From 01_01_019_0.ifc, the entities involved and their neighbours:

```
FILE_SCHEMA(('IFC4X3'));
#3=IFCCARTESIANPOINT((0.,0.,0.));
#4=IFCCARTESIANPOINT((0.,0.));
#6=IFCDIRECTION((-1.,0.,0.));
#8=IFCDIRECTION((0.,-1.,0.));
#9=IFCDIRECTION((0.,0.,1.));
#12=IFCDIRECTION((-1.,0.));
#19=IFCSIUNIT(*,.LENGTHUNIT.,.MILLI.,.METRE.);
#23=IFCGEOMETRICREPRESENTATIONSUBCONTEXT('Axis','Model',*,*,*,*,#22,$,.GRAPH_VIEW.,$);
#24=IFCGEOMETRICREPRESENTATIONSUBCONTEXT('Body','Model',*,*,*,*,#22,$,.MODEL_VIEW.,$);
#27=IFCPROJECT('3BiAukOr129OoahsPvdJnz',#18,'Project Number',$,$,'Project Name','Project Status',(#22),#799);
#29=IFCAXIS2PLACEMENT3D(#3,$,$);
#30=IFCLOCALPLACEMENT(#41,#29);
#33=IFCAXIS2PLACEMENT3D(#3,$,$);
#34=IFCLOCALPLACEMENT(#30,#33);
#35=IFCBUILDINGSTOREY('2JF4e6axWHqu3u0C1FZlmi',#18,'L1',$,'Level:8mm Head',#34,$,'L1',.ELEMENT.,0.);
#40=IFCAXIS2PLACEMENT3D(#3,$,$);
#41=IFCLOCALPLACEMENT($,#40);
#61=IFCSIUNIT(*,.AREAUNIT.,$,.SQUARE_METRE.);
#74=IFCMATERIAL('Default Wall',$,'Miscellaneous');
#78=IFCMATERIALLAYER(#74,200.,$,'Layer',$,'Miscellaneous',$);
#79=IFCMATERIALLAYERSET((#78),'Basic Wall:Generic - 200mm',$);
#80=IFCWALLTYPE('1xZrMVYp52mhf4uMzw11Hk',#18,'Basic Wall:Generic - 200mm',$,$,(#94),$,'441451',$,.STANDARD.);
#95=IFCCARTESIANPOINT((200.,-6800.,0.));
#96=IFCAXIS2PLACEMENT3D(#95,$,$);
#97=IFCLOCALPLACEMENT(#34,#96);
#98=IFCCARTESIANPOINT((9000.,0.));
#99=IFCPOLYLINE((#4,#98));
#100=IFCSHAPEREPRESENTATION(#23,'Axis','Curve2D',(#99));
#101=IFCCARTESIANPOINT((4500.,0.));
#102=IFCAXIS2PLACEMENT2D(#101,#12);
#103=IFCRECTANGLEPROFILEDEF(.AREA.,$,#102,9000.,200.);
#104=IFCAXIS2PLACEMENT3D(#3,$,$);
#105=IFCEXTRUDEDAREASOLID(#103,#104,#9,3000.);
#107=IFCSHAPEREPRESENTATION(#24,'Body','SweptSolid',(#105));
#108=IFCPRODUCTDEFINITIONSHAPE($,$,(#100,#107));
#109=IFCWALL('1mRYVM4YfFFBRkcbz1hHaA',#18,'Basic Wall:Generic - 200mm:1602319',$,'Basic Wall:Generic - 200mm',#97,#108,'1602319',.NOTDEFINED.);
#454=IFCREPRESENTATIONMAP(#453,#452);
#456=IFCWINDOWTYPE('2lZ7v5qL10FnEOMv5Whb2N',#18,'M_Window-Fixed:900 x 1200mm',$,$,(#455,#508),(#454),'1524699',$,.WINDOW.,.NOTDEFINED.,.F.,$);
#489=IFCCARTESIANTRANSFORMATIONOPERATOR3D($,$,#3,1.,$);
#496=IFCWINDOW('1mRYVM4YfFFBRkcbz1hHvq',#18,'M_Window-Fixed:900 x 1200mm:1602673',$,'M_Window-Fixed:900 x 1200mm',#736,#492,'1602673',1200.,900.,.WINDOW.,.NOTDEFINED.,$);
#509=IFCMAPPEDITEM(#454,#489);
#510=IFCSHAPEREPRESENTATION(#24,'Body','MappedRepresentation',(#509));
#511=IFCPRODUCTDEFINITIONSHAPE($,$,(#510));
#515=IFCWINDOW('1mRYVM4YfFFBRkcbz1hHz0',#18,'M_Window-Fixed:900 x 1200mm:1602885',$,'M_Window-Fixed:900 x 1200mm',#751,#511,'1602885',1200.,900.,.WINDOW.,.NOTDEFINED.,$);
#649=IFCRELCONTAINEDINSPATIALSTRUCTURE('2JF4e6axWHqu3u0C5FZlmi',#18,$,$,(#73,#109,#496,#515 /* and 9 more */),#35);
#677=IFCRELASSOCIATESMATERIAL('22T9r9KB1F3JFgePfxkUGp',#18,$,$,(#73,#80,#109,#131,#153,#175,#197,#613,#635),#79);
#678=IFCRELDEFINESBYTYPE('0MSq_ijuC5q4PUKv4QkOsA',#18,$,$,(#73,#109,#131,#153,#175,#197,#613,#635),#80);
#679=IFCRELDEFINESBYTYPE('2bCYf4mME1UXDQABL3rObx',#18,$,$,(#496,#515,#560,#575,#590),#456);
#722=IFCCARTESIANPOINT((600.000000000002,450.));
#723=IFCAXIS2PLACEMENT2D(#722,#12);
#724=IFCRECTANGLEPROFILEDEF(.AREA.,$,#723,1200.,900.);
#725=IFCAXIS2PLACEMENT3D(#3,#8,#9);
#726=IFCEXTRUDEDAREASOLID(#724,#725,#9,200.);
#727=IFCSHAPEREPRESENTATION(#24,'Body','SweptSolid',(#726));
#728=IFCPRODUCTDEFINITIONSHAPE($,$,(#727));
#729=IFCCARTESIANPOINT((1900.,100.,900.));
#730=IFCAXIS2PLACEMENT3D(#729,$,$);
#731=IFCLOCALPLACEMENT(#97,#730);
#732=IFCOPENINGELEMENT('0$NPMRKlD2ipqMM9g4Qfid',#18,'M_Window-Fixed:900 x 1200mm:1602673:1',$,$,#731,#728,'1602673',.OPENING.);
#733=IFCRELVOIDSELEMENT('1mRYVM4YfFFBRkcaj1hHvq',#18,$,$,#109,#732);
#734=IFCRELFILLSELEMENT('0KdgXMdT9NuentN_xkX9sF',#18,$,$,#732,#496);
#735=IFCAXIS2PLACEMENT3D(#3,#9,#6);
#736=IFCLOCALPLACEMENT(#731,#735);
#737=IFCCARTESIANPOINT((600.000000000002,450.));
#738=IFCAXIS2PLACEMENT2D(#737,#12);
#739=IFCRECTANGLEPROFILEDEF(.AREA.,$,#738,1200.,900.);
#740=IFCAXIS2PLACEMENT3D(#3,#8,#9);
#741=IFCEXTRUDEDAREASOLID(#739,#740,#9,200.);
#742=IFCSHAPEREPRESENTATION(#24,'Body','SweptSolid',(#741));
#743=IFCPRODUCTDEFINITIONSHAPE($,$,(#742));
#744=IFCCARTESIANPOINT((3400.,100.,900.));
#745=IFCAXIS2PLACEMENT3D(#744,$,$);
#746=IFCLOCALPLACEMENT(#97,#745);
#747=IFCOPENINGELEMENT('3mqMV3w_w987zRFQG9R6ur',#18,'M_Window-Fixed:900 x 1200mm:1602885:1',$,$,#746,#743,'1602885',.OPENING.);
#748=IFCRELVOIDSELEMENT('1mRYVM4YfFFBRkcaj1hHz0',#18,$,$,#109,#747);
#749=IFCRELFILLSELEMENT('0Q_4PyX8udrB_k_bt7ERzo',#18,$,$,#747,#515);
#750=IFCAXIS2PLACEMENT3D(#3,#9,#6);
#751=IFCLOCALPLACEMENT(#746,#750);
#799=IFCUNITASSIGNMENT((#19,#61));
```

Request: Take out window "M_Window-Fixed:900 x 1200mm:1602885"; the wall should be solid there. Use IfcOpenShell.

```python
import ifcopenshell
import ifcopenshell.api.feature
import ifcopenshell.api.root
import ifcopenshell.geom
import ifcopenshell.util.shape

model = ifcopenshell.open("01_01_019_0.ifc")
settings = ifcopenshell.geom.settings()


def volume(element):
    """Net volume in cubic metres, openings subtracted."""
    shape = ifcopenshell.geom.create_shape(settings, element)
    return ifcopenshell.util.shape.get_volume(shape.geometry)


window = model.by_id(515)
opening = window.FillsVoids[0].RelatingOpeningElement
wall = opening.VoidsElements[0].RelatingBuildingElement
before = volume(wall)

ifcopenshell.api.root.remove_product(model, product=window)
ifcopenshell.api.feature.remove_feature(model, feature=opening)

after = volume(wall)

print(f"wall volume {before:.3f} -> {after:.3f} m3")

model.write("01_01_019_0_rev.ifc")
```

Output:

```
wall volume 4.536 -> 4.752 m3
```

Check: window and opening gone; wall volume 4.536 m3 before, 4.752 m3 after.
